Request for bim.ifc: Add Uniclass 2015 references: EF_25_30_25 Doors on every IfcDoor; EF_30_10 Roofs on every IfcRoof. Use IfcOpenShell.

First a look at what the model holds.

```python
import ifcopenshell

model = ifcopenshell.open("bim.ifc")
print(model.schema)
print("classifications:", [c.Name for c in model.by_type("IfcClassification")])
for ifc_class in ("IfcDoor", "IfcRoof", "IfcStair", "IfcWall", "IfcWindow"):
    print(ifc_class, len(model.by_type(ifc_class)))
```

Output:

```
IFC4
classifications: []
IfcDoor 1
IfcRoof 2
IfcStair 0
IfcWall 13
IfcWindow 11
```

```python
import ifcopenshell
import ifcopenshell.api.classification

model = ifcopenshell.open("bim.ifc")

system = ifcopenshell.api.classification.add_classification(model, classification="Uniclass 2015")

codes = {
    "IfcDoor": ("EF_25_30_25", "Doors"),
    "IfcRoof": ("EF_30_10", "Roofs"),
}
for ifc_class, (code, name) in codes.items():
    products = model.by_type(ifc_class)
    ifcopenshell.api.classification.add_reference(
        model, products=products, classification=system, identification=code, name=name
    )
    print(code, len(products))

model.write("bim_v2.ifc")
```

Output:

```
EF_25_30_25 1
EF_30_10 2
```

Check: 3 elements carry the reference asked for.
